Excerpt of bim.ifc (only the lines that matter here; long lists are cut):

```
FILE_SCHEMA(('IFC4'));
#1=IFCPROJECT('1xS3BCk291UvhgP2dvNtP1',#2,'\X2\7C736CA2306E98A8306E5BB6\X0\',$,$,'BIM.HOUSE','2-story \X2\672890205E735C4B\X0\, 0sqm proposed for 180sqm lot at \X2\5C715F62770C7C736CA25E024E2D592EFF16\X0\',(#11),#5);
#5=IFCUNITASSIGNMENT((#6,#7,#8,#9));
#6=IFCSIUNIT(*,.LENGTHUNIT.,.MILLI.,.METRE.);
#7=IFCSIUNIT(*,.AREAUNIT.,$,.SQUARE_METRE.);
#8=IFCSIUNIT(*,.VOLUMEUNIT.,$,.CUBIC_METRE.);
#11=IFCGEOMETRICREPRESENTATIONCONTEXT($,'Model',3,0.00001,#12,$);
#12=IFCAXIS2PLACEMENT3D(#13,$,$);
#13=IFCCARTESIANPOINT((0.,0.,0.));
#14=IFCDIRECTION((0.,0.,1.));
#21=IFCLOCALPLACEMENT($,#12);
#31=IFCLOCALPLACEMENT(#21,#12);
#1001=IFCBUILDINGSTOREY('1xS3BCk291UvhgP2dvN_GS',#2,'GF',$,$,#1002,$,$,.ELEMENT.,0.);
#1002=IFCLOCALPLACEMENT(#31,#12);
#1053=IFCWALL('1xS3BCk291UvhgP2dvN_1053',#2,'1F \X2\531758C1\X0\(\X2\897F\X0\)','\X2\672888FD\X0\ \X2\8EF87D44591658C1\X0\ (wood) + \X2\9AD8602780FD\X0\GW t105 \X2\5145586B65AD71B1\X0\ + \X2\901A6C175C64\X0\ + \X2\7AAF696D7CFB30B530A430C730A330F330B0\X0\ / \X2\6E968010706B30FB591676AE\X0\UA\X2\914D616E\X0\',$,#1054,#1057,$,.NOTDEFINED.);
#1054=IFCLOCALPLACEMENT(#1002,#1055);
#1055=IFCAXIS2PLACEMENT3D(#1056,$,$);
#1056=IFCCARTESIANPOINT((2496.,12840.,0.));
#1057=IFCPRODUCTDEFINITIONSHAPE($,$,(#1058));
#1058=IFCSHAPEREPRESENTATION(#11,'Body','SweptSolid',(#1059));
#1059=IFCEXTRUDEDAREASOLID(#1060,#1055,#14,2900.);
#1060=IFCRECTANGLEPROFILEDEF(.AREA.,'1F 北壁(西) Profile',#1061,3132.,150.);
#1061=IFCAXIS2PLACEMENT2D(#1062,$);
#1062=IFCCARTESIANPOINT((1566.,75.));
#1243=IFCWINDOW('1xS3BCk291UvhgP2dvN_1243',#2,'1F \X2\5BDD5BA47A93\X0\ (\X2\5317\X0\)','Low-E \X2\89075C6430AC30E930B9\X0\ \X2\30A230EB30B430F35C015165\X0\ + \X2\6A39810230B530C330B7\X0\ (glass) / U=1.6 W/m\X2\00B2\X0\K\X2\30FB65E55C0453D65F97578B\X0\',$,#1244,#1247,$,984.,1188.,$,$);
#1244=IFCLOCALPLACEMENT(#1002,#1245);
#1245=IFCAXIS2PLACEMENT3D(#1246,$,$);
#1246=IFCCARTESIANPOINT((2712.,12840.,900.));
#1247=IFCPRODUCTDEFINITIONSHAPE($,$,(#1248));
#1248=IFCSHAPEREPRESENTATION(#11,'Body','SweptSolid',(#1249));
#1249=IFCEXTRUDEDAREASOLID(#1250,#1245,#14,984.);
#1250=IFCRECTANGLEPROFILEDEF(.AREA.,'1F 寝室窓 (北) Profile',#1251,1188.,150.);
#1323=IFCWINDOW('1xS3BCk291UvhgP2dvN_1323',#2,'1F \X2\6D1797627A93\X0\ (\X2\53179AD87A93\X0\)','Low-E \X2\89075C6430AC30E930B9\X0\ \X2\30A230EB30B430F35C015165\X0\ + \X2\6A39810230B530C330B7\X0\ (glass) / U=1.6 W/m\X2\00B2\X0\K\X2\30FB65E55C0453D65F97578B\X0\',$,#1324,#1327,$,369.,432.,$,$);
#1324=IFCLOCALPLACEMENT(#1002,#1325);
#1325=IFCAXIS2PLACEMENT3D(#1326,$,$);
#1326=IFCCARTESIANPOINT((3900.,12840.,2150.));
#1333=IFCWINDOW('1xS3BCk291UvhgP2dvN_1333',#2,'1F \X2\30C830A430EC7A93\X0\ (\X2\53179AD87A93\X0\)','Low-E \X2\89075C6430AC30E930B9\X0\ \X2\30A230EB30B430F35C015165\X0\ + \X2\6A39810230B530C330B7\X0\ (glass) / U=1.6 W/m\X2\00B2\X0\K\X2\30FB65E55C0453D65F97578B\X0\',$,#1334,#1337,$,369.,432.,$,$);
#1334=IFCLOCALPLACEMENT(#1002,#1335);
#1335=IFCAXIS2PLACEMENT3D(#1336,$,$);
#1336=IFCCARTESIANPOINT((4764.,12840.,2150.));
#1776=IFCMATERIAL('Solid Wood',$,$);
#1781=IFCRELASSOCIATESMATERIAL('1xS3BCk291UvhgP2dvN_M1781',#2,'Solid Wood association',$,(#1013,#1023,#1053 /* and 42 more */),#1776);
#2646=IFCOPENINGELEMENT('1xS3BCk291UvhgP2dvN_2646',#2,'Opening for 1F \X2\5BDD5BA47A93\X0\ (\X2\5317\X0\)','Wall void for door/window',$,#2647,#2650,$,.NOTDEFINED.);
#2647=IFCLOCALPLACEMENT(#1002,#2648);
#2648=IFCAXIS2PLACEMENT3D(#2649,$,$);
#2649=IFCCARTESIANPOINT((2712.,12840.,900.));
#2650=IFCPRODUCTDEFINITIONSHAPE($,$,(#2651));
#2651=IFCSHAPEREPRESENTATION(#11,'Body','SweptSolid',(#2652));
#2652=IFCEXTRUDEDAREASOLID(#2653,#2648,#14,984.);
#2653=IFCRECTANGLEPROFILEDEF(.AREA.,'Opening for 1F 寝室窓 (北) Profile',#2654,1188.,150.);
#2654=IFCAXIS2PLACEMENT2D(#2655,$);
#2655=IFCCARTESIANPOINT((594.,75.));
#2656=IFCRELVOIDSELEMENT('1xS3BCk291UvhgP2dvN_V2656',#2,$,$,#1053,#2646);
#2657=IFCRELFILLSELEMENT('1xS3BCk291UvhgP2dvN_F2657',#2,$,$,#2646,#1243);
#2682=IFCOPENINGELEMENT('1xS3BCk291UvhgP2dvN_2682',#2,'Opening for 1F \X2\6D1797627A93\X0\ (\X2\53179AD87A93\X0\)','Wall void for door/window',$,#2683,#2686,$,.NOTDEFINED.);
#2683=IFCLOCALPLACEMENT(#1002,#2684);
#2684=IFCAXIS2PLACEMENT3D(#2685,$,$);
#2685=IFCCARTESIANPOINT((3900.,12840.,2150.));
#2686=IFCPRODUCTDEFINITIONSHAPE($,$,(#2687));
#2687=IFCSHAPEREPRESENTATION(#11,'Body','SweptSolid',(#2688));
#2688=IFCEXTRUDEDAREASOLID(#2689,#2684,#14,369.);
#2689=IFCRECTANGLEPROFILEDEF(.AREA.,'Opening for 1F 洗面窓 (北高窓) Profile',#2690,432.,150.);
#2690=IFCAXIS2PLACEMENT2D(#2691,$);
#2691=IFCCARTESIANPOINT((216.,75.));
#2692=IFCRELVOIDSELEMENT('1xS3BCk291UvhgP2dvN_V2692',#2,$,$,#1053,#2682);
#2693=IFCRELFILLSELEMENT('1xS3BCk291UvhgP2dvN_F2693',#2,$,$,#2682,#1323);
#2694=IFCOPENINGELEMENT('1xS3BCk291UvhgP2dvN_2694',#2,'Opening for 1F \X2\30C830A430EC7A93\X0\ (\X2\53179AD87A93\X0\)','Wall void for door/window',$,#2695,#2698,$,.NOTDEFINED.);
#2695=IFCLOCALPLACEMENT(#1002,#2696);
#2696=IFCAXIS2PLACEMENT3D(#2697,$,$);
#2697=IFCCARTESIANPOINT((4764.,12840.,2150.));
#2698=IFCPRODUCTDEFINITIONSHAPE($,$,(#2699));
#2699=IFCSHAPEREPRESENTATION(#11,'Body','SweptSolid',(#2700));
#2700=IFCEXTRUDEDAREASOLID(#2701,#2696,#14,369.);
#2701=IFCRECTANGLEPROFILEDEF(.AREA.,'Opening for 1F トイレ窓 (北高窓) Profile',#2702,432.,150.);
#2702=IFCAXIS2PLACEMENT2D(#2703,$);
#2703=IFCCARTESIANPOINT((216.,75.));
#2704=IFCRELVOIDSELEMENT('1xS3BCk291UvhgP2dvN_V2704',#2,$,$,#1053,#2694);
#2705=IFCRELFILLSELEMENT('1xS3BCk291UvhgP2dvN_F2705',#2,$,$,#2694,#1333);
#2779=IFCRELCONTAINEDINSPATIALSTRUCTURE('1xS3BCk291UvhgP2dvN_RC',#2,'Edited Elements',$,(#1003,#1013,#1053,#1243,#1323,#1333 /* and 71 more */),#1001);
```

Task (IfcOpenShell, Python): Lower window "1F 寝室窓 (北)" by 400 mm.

```python
import numpy as np
import ifcopenshell
import ifcopenshell.api.geometry
import ifcopenshell.util.placement
import ifcopenshell.util.unit

model = ifcopenshell.open("bim.ifc")
unit_scale = ifcopenshell.util.unit.calculate_unit_scale(model)

window = model.by_id(1243)
opening = window.FillsVoids[0].RelatingOpeningElement
dz = -400.0

shift = np.array([0.0, 0.0, dz])
# The window is not placed relative to its opening, so move both.
for product in (opening, window):
    matrix = ifcopenshell.util.placement.get_local_placement(product.ObjectPlacement)
    matrix[:3, 3] += shift
    ifcopenshell.api.geometry.edit_object_placement(model, product=product, matrix=matrix, is_si=False)

print(f"moved by {dz * unit_scale:+.3f} m")

model.write("bim_updated.ifc")
```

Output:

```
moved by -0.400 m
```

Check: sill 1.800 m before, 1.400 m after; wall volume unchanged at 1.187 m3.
